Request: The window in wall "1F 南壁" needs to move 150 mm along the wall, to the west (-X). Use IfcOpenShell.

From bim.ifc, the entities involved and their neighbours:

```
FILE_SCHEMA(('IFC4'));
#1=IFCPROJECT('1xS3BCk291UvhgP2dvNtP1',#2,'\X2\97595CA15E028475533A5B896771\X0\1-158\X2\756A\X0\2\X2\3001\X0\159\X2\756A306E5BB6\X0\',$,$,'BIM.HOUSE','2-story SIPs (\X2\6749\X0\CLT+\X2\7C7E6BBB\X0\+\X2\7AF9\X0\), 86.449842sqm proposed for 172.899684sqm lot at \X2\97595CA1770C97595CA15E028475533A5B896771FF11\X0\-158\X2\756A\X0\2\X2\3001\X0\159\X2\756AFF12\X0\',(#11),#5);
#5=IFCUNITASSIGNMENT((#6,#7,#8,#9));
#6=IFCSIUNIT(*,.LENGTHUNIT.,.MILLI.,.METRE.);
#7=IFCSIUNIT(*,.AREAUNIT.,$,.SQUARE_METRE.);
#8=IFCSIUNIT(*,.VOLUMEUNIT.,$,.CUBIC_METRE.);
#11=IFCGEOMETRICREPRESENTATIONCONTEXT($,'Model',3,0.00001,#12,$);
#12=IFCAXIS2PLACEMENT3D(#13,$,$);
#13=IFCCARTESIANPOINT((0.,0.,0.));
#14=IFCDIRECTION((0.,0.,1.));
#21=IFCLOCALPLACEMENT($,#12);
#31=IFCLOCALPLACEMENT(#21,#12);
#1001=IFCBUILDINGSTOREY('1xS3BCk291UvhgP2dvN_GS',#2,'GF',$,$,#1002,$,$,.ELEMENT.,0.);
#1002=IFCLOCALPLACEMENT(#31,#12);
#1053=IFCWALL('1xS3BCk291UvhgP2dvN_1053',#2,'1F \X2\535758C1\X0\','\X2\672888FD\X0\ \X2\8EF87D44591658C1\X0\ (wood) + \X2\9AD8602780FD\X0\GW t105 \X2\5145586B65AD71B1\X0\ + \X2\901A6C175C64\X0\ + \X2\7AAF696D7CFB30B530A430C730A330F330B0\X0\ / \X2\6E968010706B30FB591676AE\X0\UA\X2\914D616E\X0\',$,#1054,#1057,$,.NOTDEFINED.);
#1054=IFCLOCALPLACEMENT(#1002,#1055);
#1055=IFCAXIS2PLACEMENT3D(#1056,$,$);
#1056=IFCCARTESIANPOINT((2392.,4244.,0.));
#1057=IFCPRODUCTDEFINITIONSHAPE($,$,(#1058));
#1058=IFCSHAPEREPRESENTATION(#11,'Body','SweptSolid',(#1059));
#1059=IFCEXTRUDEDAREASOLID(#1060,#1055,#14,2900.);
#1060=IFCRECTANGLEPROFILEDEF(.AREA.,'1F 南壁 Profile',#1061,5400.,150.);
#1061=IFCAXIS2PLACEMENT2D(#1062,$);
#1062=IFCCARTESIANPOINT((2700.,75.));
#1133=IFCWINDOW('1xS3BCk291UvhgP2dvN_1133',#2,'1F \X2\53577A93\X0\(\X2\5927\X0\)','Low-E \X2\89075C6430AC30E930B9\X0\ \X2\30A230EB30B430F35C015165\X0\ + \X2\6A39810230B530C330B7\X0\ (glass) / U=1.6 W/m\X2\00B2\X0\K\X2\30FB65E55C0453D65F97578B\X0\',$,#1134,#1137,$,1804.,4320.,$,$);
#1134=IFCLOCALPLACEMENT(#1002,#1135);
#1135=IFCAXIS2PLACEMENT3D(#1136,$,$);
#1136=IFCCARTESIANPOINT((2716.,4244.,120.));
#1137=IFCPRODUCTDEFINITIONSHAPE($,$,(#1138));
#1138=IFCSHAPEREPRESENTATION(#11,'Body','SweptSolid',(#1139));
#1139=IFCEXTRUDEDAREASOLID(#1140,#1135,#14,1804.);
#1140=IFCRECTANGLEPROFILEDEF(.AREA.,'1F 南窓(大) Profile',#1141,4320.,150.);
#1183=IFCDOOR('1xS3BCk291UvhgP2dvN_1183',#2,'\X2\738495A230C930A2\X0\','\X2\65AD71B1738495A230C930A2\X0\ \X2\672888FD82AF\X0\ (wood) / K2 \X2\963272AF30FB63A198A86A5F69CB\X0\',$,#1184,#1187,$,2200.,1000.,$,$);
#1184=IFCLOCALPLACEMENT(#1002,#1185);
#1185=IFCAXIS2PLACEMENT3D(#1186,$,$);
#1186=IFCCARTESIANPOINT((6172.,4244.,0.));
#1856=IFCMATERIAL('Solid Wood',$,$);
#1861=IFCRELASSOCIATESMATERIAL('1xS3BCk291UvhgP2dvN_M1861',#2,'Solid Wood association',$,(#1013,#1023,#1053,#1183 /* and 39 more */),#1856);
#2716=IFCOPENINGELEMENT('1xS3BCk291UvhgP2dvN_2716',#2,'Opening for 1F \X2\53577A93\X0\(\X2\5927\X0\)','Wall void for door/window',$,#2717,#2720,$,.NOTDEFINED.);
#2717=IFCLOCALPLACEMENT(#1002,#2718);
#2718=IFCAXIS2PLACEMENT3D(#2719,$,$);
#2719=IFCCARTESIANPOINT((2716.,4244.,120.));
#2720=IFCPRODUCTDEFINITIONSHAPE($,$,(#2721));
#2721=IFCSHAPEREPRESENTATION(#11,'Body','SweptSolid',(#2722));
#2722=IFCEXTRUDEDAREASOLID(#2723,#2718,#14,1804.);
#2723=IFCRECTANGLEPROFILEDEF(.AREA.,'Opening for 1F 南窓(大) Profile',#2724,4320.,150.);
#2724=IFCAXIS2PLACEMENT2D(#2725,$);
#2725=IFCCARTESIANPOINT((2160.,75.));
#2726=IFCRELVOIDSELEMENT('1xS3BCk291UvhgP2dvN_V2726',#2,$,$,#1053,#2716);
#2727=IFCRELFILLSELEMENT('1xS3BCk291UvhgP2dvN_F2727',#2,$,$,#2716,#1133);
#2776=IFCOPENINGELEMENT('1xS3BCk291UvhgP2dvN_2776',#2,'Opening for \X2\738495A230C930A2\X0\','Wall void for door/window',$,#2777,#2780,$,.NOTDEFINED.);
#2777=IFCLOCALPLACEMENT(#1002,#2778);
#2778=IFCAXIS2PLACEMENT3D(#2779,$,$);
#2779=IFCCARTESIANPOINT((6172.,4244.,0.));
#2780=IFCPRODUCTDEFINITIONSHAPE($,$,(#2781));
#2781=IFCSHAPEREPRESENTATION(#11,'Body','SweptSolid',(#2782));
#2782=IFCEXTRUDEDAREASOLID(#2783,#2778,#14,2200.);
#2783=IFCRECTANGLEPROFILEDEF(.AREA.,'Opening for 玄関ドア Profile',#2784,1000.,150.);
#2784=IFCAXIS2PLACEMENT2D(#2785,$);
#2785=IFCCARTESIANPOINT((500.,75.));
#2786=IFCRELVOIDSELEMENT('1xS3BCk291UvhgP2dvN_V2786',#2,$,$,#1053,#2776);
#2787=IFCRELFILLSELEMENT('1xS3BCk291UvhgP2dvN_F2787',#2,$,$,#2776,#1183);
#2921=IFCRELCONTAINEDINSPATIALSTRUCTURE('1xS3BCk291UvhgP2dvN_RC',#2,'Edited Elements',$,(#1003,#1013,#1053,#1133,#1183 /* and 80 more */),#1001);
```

```python
import ifcopenshell
import ifcopenshell.api.geometry
import ifcopenshell.util.placement

model = ifcopenshell.open("bim.ifc")

window = model.by_id(1133)
opening = window.FillsVoids[0].RelatingOpeningElement
wall = opening.VoidsElements[0].RelatingBuildingElement

wall_matrix = ifcopenshell.util.placement.get_local_placement(wall.ObjectPlacement)
shift = wall_matrix[:3, 0] * -150.0
before = ifcopenshell.util.placement.get_local_placement(window.ObjectPlacement)[:3, 3].copy()

# The window is not placed relative to its opening, so move both.
for product in (opening, window):
    matrix = ifcopenshell.util.placement.get_local_placement(product.ObjectPlacement)
    matrix[:3, 3] += shift
    ifcopenshell.api.geometry.edit_object_placement(model, product=product, matrix=matrix, is_si=False)

after = ifcopenshell.util.placement.get_local_placement(window.ObjectPlacement)[:3, 3]
print("window moved by", (after - before).round(3) + 0.0)

model.write("bim_rev.ifc")
```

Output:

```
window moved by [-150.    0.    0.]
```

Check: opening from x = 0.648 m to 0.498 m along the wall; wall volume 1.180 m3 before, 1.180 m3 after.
